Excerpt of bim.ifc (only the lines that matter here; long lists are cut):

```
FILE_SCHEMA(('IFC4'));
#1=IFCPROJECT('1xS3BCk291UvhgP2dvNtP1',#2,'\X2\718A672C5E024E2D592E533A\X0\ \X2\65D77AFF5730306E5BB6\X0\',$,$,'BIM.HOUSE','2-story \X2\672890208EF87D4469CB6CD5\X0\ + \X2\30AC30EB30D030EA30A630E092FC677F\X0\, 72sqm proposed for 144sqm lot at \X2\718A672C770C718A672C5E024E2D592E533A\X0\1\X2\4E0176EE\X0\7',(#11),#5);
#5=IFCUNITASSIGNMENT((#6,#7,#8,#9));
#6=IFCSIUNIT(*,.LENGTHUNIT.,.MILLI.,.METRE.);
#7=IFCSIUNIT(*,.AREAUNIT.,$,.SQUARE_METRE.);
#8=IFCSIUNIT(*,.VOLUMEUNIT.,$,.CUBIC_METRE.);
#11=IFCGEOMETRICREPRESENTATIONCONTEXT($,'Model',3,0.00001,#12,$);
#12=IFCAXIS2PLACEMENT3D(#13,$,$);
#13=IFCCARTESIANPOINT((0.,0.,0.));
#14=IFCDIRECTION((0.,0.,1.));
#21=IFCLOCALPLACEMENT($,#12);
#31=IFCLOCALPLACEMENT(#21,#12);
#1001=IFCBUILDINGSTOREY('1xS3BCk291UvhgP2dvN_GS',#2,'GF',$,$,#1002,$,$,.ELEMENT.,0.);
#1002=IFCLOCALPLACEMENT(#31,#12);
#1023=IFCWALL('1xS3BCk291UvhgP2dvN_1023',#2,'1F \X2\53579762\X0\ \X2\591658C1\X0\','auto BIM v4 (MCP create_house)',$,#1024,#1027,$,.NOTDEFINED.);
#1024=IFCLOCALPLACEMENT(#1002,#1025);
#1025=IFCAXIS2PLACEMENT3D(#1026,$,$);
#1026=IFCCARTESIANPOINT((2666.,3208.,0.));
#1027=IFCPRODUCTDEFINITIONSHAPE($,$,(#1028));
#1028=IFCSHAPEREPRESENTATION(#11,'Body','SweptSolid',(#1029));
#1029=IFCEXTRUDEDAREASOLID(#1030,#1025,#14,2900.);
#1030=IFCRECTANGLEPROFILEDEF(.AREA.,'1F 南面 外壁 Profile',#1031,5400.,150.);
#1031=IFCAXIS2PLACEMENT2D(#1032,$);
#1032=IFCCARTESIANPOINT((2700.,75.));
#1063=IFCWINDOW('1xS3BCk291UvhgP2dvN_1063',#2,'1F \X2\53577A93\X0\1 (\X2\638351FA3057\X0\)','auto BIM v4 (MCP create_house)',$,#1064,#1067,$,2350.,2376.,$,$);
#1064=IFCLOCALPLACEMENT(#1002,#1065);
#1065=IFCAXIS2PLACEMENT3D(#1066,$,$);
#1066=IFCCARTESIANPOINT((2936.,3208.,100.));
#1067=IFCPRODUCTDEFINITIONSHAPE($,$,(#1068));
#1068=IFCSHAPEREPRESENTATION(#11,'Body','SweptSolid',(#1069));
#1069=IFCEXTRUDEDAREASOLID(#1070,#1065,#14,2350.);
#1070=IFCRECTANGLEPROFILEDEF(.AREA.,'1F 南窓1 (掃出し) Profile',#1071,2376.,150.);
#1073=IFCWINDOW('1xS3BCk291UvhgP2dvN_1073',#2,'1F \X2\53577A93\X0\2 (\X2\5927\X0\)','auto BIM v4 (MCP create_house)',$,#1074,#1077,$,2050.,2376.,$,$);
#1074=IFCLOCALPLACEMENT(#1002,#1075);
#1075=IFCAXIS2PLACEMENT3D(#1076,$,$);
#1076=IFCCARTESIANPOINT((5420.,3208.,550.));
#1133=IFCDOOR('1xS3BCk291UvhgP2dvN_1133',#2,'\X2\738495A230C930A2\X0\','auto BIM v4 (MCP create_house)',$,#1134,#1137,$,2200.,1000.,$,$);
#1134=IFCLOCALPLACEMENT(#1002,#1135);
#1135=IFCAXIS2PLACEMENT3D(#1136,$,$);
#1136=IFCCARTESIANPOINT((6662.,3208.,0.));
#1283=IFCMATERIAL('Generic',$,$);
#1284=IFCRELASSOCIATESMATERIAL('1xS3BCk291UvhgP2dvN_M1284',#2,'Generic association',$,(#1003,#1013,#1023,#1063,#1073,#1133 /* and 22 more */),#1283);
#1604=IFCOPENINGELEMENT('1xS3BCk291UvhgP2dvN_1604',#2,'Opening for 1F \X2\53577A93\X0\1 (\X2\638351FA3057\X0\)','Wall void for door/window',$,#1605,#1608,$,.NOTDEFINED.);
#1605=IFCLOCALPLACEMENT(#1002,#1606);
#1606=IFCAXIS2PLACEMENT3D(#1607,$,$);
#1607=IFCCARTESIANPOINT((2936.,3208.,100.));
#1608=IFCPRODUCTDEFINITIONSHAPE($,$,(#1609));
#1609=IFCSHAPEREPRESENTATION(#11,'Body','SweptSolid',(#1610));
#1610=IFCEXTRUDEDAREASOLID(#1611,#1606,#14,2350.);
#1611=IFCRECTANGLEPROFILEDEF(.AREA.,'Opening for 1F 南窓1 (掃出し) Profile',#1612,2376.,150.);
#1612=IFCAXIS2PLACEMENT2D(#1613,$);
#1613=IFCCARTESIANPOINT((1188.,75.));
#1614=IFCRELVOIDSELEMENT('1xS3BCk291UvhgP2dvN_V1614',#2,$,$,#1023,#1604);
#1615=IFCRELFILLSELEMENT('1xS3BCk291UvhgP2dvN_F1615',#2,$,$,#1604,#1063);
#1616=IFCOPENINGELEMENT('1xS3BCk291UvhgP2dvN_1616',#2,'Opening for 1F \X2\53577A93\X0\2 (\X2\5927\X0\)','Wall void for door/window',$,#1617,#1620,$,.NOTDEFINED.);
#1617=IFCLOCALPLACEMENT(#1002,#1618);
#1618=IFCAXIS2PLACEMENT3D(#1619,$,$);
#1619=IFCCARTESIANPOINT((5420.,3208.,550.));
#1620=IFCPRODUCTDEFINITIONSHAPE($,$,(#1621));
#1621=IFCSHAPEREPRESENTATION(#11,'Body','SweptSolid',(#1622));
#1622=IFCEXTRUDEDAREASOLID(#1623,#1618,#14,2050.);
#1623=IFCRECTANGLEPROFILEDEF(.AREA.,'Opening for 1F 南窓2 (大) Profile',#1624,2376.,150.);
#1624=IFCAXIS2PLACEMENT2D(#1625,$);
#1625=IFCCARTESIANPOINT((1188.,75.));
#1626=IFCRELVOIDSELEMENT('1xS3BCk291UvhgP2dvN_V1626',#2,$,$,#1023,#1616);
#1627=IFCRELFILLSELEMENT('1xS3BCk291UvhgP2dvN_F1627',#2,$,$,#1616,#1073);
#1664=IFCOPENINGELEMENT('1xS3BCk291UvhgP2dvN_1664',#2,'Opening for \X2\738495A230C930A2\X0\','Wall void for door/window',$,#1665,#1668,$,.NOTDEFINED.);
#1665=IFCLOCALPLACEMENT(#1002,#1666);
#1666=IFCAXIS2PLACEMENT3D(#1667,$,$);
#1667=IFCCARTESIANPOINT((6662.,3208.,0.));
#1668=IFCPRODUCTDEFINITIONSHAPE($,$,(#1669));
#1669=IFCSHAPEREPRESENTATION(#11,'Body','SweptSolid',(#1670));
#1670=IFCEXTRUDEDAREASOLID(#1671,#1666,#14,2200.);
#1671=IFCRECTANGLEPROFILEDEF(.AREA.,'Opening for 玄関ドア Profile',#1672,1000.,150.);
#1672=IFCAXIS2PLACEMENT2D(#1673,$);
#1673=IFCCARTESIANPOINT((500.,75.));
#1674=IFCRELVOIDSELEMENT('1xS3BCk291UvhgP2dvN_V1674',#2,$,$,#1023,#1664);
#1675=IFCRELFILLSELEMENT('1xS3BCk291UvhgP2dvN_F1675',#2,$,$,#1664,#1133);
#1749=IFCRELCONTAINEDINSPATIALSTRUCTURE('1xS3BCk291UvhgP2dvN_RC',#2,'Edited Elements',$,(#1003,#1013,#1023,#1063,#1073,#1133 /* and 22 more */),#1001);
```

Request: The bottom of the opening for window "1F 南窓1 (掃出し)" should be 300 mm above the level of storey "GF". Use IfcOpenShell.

```python
import numpy as np
import ifcopenshell
import ifcopenshell.api.geometry
import ifcopenshell.geom
import ifcopenshell.util.element
import ifcopenshell.util.placement
import ifcopenshell.util.shape
import ifcopenshell.util.unit

model = ifcopenshell.open("bim.ifc")
unit_scale = ifcopenshell.util.unit.calculate_unit_scale(model)

window = model.by_guid("1xS3BCk291UvhgP2dvN_1063")
opening = window.FillsVoids[0].RelatingOpeningElement
storey = ifcopenshell.util.element.get_container(window, ifc_class="IfcBuildingStorey")
level = ifcopenshell.util.placement.get_local_placement(storey.ObjectPlacement)[2, 3]

# The opening's origin need not be at the sill, so measure its lowest point.
shape = ifcopenshell.geom.create_shape(ifcopenshell.geom.settings(), opening)
bottom = ifcopenshell.util.shape.get_shape_bottom_elevation(shape, shape.geometry) / unit_scale
dz = level + 300.0 - bottom

shift = np.array([0.0, 0.0, dz])
# The window is not placed relative to its opening, so move both.
for product in (opening, window):
    matrix = ifcopenshell.util.placement.get_local_placement(product.ObjectPlacement)
    matrix[:3, 3] += shift
    ifcopenshell.api.geometry.edit_object_placement(model, product=product, matrix=matrix, is_si=False)

print(f"moved by {dz * unit_scale:+.3f} m")

model.write("bim_rev.ifc")
```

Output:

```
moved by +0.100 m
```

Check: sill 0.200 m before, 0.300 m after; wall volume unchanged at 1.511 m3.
